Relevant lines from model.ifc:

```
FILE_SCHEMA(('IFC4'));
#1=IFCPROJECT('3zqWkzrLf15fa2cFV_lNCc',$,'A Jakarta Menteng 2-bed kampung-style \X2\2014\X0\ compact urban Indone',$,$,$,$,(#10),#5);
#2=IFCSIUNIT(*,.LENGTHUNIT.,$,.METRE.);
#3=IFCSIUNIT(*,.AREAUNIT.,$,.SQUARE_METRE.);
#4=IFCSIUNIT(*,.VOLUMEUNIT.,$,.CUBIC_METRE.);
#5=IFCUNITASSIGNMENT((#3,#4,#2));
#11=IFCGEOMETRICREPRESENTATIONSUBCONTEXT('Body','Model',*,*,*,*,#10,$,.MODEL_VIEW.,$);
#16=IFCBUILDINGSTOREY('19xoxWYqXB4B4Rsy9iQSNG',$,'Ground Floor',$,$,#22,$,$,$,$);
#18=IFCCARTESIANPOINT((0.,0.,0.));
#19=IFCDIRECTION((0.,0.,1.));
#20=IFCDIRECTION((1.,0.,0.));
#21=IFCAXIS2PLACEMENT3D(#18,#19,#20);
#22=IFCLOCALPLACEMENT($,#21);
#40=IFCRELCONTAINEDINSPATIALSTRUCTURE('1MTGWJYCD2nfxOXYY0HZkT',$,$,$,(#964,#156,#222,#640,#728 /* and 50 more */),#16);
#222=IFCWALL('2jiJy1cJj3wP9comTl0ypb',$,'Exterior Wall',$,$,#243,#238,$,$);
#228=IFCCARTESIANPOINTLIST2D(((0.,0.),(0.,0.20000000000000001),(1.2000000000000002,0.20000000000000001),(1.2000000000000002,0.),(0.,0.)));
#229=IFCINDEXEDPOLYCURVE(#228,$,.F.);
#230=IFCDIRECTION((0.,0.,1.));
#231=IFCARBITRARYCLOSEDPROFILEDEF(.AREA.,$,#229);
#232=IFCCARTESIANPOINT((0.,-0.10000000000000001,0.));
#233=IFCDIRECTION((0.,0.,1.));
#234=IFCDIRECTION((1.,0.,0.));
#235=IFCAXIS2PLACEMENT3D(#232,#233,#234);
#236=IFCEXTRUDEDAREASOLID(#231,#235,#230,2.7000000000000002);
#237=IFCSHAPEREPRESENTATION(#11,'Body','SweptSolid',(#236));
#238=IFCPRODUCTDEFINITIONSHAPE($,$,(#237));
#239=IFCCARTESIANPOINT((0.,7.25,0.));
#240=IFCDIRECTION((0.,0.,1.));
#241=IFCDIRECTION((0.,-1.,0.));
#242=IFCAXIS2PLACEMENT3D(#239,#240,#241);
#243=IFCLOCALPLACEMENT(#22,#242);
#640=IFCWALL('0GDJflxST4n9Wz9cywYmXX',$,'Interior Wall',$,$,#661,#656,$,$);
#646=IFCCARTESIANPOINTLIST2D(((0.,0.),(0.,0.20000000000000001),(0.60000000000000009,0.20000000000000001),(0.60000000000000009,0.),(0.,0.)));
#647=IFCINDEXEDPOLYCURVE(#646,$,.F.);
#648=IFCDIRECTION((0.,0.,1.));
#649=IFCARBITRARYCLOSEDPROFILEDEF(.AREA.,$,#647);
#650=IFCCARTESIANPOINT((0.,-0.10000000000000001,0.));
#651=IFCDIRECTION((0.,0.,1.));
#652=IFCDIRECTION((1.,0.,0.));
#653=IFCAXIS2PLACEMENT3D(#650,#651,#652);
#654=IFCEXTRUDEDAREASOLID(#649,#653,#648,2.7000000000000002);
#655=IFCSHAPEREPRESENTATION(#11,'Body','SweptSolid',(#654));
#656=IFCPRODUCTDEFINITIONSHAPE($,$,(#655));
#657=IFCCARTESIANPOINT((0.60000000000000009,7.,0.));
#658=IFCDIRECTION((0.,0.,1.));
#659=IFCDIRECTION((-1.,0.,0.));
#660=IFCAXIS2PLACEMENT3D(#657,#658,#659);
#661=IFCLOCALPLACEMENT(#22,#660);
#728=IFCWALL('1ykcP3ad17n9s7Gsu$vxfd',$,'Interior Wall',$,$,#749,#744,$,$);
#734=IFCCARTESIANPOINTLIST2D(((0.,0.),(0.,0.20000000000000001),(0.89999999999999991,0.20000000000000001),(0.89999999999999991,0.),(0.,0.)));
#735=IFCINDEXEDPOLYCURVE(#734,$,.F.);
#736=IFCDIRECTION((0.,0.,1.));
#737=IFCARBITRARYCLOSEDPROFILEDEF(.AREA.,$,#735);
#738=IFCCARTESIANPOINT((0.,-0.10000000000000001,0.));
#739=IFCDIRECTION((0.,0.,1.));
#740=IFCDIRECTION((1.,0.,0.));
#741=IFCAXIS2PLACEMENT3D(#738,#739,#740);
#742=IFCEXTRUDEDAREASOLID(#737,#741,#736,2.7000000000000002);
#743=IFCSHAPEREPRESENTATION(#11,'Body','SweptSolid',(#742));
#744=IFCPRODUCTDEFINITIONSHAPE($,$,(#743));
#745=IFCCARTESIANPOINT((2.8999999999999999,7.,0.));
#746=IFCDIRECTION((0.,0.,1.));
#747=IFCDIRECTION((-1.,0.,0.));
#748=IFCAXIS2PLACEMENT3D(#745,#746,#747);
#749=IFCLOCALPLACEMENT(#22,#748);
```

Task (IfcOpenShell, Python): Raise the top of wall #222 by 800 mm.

```python
import ifcopenshell
import ifcopenshell.geom
import ifcopenshell.util.representation
import ifcopenshell.util.shape
import ifcopenshell.util.unit

model = ifcopenshell.open("model.ifc")
unit_scale = ifcopenshell.util.unit.calculate_unit_scale(model)
settings = ifcopenshell.geom.settings()


def volume(element):
    """Net volume in cubic metres, openings subtracted."""
    shape = ifcopenshell.geom.create_shape(settings, element)
    return ifcopenshell.util.shape.get_volume(shape.geometry)


wall = model.by_guid("2jiJy1cJj3wP9comTl0ypb")
before = volume(wall)

body = ifcopenshell.util.representation.get_representation(wall, "Model", "Body")
solid = body.Items[0]
old_height = solid.Depth
solid.Depth += 0.8 / unit_scale
after = volume(wall)

print(f"height {old_height:g} -> {solid.Depth:g}, volume {before:.3f} -> {after:.3f} m3")

model.write("model_v2.ifc")
```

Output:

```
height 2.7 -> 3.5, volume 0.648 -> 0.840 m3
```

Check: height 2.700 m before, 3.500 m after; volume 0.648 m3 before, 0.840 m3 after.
